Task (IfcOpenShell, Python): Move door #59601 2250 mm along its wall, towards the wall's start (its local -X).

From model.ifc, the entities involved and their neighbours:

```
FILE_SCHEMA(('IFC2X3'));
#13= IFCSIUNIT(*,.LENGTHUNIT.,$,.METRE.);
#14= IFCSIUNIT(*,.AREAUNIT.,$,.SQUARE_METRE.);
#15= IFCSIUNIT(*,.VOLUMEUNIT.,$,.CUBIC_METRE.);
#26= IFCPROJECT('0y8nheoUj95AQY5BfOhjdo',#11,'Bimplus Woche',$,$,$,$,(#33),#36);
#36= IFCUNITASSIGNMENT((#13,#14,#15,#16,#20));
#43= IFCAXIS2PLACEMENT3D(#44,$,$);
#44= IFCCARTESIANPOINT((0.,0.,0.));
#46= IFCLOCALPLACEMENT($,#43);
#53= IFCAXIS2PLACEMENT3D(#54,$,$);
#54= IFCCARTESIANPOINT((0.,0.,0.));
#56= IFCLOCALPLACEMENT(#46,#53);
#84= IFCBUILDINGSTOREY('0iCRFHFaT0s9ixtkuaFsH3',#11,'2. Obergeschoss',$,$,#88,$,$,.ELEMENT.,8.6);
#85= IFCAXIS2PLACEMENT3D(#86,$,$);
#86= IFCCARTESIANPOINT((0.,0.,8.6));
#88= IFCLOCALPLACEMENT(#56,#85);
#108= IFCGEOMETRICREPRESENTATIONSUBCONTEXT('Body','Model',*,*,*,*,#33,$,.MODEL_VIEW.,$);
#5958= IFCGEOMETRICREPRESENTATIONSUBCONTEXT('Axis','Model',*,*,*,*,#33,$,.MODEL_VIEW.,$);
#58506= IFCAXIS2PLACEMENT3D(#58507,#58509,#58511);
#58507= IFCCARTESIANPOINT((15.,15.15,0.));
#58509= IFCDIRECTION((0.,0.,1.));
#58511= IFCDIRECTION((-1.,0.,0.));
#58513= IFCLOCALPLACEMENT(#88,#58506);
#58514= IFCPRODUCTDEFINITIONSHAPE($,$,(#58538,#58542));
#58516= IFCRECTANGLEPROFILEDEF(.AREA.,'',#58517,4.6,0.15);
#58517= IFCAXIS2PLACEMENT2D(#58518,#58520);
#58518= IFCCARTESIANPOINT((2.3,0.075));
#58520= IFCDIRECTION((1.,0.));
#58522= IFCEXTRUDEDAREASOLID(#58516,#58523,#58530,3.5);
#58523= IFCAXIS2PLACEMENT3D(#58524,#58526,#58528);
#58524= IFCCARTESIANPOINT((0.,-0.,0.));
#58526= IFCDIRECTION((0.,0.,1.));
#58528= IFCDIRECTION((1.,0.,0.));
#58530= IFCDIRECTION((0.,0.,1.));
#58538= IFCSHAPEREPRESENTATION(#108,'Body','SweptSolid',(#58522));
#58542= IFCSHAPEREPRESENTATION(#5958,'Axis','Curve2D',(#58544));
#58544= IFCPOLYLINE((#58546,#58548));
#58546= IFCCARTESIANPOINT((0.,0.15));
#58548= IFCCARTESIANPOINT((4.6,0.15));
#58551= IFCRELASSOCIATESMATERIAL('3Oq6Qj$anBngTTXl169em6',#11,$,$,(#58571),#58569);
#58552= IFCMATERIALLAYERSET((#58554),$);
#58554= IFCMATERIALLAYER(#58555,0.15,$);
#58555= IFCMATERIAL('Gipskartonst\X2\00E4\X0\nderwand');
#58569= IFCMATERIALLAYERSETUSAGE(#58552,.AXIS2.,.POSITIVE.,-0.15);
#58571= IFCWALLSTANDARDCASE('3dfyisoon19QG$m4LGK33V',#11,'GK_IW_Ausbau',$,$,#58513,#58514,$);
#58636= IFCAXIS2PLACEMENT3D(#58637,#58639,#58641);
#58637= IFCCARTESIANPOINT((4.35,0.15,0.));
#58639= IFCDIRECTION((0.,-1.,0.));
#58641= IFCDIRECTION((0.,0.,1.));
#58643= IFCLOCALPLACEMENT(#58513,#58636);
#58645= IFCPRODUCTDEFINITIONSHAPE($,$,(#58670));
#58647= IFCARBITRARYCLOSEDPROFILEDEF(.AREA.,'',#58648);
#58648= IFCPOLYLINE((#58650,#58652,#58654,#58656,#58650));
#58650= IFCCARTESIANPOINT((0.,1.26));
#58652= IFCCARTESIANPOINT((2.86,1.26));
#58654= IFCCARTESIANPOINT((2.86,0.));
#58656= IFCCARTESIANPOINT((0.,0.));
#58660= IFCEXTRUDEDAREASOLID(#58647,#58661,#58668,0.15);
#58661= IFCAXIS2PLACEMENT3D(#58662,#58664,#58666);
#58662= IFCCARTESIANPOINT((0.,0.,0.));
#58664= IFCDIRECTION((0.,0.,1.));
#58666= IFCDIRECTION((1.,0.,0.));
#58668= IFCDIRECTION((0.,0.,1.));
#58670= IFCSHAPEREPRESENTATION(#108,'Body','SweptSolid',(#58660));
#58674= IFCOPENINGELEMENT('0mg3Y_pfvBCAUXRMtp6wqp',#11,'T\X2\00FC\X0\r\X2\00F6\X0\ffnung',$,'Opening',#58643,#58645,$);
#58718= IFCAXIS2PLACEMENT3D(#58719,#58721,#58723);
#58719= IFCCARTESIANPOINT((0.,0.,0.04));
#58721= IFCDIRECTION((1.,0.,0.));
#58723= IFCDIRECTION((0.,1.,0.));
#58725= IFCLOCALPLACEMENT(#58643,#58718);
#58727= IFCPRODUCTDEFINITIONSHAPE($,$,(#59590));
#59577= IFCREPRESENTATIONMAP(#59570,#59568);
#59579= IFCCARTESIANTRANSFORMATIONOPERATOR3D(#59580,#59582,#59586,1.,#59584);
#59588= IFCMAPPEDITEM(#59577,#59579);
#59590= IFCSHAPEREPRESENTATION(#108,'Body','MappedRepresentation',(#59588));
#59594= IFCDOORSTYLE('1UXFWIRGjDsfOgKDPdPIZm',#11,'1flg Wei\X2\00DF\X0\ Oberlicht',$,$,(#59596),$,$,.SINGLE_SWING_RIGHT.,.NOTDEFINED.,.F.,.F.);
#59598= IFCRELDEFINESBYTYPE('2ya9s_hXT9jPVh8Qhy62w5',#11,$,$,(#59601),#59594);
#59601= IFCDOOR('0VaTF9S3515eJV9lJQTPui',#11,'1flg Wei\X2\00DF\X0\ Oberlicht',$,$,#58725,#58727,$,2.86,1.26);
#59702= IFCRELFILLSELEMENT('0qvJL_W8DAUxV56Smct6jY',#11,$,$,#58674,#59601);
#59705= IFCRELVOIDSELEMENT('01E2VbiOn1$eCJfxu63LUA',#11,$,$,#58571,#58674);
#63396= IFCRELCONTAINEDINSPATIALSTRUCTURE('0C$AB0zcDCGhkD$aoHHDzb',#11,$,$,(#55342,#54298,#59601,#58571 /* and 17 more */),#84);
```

```python
import ifcopenshell
import ifcopenshell.api.geometry
import ifcopenshell.util.placement
import ifcopenshell.util.unit

model = ifcopenshell.open("model.ifc")
unit_scale = ifcopenshell.util.unit.calculate_unit_scale(model)

door = model.by_id(59601)
opening = door.FillsVoids[0].RelatingOpeningElement
wall = opening.VoidsElements[0].RelatingBuildingElement

wall_matrix = ifcopenshell.util.placement.get_local_placement(wall.ObjectPlacement)
shift = wall_matrix[:3, 0] * -2.25 / unit_scale
before = ifcopenshell.util.placement.get_local_placement(door.ObjectPlacement)[:3, 3].copy()

# The door is placed relative to its opening, so it follows when the opening moves.
matrix = ifcopenshell.util.placement.get_local_placement(opening.ObjectPlacement)
matrix[:3, 3] += shift
ifcopenshell.api.geometry.edit_object_placement(
    model, product=opening, matrix=matrix, is_si=False, should_transform_children=True
)

after = ifcopenshell.util.placement.get_local_placement(door.ObjectPlacement)[:3, 3]
print("door moved by", (after - before).round(3) + 0.0)

model.write("model_v2.ifc")
```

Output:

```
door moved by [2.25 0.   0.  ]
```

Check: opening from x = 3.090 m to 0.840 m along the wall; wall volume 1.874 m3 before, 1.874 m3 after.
